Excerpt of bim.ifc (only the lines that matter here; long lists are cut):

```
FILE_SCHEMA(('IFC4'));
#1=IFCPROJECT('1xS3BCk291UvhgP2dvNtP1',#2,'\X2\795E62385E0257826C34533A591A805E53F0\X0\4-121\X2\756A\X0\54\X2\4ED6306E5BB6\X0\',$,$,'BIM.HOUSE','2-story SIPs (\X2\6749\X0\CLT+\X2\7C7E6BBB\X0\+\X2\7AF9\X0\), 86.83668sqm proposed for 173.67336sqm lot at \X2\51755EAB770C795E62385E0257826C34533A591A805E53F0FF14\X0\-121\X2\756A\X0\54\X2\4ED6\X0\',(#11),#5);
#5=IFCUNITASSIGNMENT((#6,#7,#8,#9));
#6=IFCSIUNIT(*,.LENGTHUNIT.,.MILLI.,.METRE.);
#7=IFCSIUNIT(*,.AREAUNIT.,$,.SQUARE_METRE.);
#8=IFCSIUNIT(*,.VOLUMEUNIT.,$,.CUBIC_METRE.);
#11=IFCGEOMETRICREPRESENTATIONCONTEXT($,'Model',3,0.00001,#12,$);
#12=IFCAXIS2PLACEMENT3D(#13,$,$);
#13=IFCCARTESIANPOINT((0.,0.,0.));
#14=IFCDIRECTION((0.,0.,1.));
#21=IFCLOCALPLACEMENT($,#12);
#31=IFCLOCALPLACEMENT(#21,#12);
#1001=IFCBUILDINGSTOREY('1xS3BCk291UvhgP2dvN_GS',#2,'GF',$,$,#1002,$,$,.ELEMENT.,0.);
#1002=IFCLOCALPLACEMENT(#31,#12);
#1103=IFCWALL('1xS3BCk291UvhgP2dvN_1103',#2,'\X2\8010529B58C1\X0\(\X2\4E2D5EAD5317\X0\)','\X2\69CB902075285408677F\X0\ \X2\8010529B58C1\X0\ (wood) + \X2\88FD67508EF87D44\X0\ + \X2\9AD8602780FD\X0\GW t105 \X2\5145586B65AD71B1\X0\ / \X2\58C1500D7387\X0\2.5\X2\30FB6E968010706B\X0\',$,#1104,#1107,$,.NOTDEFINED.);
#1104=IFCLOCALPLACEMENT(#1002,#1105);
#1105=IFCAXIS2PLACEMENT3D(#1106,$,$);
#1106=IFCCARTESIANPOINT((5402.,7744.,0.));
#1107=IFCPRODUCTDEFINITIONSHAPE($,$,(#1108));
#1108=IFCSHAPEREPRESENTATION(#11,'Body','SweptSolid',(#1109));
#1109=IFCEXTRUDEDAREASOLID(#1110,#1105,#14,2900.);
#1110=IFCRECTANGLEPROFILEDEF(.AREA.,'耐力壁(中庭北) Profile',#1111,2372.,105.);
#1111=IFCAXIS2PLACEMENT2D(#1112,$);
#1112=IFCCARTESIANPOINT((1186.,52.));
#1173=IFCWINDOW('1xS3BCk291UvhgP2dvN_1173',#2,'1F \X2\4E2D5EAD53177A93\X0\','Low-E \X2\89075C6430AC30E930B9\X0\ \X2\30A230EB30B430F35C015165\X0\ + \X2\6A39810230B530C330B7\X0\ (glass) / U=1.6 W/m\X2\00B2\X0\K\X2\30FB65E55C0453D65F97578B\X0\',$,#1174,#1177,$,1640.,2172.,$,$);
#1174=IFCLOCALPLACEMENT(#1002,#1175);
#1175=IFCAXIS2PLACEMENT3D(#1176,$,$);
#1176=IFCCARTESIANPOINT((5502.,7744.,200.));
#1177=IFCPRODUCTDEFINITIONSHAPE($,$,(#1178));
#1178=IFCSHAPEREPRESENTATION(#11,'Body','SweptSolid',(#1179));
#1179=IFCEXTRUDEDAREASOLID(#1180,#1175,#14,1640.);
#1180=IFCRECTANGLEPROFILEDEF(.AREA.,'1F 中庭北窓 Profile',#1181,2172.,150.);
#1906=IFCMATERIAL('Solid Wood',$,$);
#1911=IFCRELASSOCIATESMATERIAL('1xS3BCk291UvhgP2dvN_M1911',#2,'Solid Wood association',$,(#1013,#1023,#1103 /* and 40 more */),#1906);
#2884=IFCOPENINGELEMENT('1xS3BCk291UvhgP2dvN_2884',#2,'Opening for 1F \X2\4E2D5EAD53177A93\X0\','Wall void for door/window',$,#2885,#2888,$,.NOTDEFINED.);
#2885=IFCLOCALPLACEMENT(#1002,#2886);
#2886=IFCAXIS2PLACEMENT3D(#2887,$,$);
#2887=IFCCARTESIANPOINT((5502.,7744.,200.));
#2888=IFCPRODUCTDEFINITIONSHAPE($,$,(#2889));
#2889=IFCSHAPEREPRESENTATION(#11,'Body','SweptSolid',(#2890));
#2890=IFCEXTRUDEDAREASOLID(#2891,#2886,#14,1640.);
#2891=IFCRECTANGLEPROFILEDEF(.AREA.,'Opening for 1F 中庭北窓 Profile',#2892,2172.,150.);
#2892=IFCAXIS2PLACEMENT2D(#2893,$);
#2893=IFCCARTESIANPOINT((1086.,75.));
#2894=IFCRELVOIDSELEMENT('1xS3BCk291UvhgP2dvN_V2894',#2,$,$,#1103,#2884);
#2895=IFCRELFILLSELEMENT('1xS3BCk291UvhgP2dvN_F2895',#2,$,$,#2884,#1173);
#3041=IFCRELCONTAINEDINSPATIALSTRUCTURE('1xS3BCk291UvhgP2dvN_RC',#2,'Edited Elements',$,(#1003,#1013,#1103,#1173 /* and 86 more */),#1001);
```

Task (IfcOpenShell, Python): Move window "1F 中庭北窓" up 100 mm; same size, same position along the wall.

```python
import numpy as np
import ifcopenshell
import ifcopenshell.api.geometry
import ifcopenshell.util.placement
import ifcopenshell.util.unit

model = ifcopenshell.open("bim.ifc")
unit_scale = ifcopenshell.util.unit.calculate_unit_scale(model)

window = model.by_guid("1xS3BCk291UvhgP2dvN_1173")
opening = window.FillsVoids[0].RelatingOpeningElement
dz = 0.1 / unit_scale

shift = np.array([0.0, 0.0, dz])
# The window is not placed relative to its opening, so move both.
for product in (opening, window):
    matrix = ifcopenshell.util.placement.get_local_placement(product.ObjectPlacement)
    matrix[:3, 3] += shift
    ifcopenshell.api.geometry.edit_object_placement(model, product=product, matrix=matrix, is_si=False)

print(f"moved by {dz * unit_scale:+.3f} m")

model.write("bim_edited.ifc")
```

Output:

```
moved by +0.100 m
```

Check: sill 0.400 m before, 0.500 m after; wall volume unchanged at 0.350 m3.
